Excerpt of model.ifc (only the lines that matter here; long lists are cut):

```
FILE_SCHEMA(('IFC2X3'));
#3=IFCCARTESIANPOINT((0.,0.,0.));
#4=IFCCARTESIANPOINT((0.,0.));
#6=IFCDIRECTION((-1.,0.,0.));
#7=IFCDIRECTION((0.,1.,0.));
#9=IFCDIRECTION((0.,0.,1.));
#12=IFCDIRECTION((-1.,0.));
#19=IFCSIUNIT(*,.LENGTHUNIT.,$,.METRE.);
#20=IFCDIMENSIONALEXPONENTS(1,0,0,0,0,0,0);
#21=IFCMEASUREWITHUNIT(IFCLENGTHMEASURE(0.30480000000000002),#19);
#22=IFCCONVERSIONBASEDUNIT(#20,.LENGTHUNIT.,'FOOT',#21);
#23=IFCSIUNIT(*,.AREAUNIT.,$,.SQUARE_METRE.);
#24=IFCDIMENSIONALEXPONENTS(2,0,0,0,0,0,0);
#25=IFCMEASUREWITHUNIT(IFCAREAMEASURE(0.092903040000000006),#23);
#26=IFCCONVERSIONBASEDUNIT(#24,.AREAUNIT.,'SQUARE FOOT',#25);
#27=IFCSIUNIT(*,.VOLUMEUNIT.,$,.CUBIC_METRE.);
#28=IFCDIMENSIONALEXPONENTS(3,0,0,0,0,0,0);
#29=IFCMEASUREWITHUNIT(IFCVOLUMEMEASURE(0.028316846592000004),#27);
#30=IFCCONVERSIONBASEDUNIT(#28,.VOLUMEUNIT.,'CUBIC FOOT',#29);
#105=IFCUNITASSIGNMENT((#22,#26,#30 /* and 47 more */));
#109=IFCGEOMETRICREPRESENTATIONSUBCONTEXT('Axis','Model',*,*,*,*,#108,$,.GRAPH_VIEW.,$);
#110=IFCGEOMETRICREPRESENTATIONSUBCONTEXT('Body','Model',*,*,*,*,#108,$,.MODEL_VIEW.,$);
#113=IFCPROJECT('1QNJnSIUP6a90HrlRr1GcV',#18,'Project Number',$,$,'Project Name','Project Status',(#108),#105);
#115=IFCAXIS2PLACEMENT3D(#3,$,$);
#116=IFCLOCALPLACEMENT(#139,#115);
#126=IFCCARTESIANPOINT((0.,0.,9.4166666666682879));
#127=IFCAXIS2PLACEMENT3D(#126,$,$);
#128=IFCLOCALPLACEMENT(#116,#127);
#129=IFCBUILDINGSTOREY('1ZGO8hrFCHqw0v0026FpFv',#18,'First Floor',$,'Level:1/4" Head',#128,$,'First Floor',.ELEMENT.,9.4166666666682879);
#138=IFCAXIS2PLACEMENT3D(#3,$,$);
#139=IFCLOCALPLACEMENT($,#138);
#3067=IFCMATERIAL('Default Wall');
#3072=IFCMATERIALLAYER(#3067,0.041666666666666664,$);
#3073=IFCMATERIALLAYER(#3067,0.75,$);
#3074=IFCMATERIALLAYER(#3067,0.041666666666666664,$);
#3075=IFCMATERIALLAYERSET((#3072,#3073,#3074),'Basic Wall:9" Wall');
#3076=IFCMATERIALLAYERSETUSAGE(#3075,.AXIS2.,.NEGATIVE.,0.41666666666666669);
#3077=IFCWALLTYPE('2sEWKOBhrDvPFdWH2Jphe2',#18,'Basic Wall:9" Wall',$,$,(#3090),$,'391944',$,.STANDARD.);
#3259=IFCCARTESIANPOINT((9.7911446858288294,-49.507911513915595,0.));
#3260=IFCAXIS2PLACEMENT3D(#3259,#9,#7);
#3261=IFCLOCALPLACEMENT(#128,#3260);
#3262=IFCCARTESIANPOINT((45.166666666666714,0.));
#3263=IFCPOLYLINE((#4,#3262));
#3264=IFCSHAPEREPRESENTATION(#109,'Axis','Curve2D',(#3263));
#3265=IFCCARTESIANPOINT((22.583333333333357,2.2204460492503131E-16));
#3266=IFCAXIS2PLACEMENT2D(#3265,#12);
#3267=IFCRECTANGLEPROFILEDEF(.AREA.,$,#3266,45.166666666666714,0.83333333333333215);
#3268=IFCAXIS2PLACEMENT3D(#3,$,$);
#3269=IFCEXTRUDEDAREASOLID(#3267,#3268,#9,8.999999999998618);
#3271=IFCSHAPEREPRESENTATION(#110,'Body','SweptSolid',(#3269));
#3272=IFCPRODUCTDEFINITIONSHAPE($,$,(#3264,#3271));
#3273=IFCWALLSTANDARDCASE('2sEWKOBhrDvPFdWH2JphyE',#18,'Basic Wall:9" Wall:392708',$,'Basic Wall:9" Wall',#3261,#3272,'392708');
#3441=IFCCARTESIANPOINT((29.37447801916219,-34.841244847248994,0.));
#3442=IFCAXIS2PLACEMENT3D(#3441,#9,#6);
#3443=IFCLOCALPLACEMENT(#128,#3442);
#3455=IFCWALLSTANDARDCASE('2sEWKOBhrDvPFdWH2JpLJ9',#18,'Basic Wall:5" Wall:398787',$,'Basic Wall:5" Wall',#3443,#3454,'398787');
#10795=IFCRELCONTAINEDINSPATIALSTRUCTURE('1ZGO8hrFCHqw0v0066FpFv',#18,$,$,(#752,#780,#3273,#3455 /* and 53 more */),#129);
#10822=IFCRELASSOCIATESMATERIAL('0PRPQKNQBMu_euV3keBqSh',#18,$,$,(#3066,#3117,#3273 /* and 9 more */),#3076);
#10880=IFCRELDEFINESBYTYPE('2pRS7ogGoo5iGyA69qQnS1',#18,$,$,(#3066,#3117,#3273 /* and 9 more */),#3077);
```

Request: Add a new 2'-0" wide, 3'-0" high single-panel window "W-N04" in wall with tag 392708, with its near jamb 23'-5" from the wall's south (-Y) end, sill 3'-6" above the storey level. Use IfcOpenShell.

```python
import numpy as np
import ifcopenshell
import ifcopenshell.api.feature
import ifcopenshell.api.geometry
import ifcopenshell.api.root
import ifcopenshell.api.spatial
import ifcopenshell.api.type
import ifcopenshell.geom
import ifcopenshell.util.element
import ifcopenshell.util.placement
import ifcopenshell.util.representation
import ifcopenshell.util.shape
import ifcopenshell.util.unit

model = ifcopenshell.open("model.ifc")
unit_scale = ifcopenshell.util.unit.calculate_unit_scale(model)
settings = ifcopenshell.geom.settings()


def volume(element):
    """Net volume in cubic metres, openings subtracted."""
    shape = ifcopenshell.geom.create_shape(settings, element)
    return ifcopenshell.util.shape.get_volume(shape.geometry)


wall = model.by_guid("2sEWKOBhrDvPFdWH2JphyE")
storey = ifcopenshell.util.element.get_container(wall, ifc_class="IfcBuildingStorey")
context = ifcopenshell.util.representation.get_context(model, "Model", "Body", "MODEL_VIEW")
before = volume(wall)

width, height, from_end, sill = 0.6096, 0.9144, 7.1374, 1.0668  # metres

# The wall runs along its own X axis, and the end named is its -X end.
wall_shape = ifcopenshell.geom.create_shape(settings, wall)
x, y, z = ifcopenshell.util.shape.get_vertices(wall_shape.geometry).T
start = x.min() + from_end
face, thickness = float(y.min()), float(y.max() - y.min())
wall_matrix = ifcopenshell.util.placement.get_local_placement(wall.ObjectPlacement)
level = ifcopenshell.util.placement.get_local_placement(storey.ObjectPlacement)[2, 3]


def in_wall(x, y):
    """Placement at x, y metres in the wall's axes, at sill height."""
    matrix = wall_matrix.copy()
    matrix[:, 3] = wall_matrix @ np.array([x / unit_scale, y / unit_scale, 0.0, 1.0])
    matrix[2, 3] = level + sill / unit_scale
    return matrix


# Opening: a box that overshoots both wall faces by 50 mm.
opening = ifcopenshell.api.root.create_entity(model, ifc_class="IfcOpeningElement")
box = ifcopenshell.api.geometry.add_wall_representation(
    model, context=context, length=width, height=height, thickness=thickness + 0.1
)
ifcopenshell.api.geometry.assign_representation(model, product=opening, representation=box)
ifcopenshell.api.geometry.edit_object_placement(model, product=opening, matrix=in_wall(start, face - 0.05), is_si=False)
ifcopenshell.api.feature.add_feature(model, feature=opening, element=wall)

window = ifcopenshell.api.root.create_entity(model, ifc_class="IfcWindow", name="W-N04")
window.OverallWidth, window.OverallHeight = width / unit_scale, height / unit_scale
body = ifcopenshell.api.geometry.add_window_representation(
    model,
    context=context,
    overall_width=window.OverallWidth,
    overall_height=window.OverallHeight,
    partition_type="SINGLE_PANEL",
)
ifcopenshell.api.geometry.assign_representation(model, product=window, representation=body)
ifcopenshell.api.spatial.assign_container(model, products=[window], relating_structure=storey)
fills = ifcopenshell.api.feature.add_filling(model, opening=opening, element=window)
fills.OwnerHistory = window.OwnerHistory  # required in IFC2X3

# IFC2X3 keeps the operation on the window style.
style = ifcopenshell.api.root.create_entity(model, ifc_class="IfcWindowStyle", name="W-N04")
style.OperationType, style.ConstructionType = "SINGLE_PANEL", "NOTDEFINED"
style.ParameterTakesPrecedence = style.Sizeable = False
ifcopenshell.api.type.assign_type(model, related_objects=[window], relating_type=style)

# Centre the window in the wall's thickness.
ifcopenshell.api.geometry.edit_object_placement(model, product=window, matrix=in_wall(start, face), is_si=False)
window_shape = ifcopenshell.geom.create_shape(settings, window)
depth = ifcopenshell.util.shape.get_vertices(window_shape.geometry)[:, 1]
offset = face + thickness / 2 - (depth.min() + depth.max()) / 2
ifcopenshell.api.geometry.edit_object_placement(model, product=window, matrix=in_wall(start, offset), is_si=False)

after = volume(wall)

print(f"wall volume {before:.3f} -> {after:.3f} m3")

model.write("model_edited.ifc")
```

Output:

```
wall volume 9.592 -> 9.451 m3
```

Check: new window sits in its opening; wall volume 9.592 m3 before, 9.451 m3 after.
